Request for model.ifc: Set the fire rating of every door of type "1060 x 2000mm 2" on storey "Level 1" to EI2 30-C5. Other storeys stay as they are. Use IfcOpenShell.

First a look at what the model holds.

```python
import ifcopenshell
import ifcopenshell.util.element

model = ifcopenshell.open("model.ifc")
print(model.schema)
storey = next(s for s in model.by_type("IfcBuildingStorey") if s.Name == "Level 1")
doors = [e for e in ifcopenshell.util.element.get_decomposition(storey) if e.is_a("IfcDoor")]
seen = {}
for e in doors:
    element_type = ifcopenshell.util.element.get_type(e)
    key = (element_type.Name if element_type != e and element_type else None, ifcopenshell.util.element.get_pset(e, "Pset_DoorCommon", "FireRating"))
    seen[key] = seen.get(key, 0) + 1
for (name, value), count in sorted(seen.items(), key=str):
    print(count, "x", name, "|", value)
```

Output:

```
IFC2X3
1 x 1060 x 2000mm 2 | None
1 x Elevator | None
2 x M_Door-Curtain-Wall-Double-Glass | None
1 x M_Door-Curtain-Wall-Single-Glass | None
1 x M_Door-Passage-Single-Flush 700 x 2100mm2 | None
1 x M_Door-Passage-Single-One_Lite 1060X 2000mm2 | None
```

```python
import ifcopenshell
import ifcopenshell.api.pset
import ifcopenshell.util.element

model = ifcopenshell.open("model.ifc")

storey = next(s for s in model.by_type("IfcBuildingStorey") if s.Name == "Level 1")
doors = [e for e in ifcopenshell.util.element.get_decomposition(storey) if e.is_a("IfcDoor")]

count = 0
for e in doors:
    element_type = ifcopenshell.util.element.get_type(e)
    if element_type in (None, e) or element_type.Name != "1060 x 2000mm 2":
        continue
    # add_pset returns the element's existing set when there is one.
    pset = ifcopenshell.api.pset.add_pset(model, product=e, name="Pset_DoorCommon")
    ifcopenshell.api.pset.edit_pset(model, pset=pset, properties={"FireRating": "EI2 30-C5"})
    count += 1

print(count, "doors updated")

model.write("model_updated.ifc")
```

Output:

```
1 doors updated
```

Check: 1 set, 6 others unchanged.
